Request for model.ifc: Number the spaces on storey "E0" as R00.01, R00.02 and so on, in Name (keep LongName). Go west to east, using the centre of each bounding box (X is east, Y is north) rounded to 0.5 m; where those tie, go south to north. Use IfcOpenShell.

First a look at what the model holds.

```python
import ifcopenshell
import ifcopenshell.util.element
import ifcopenshell.util.placement

model = ifcopenshell.open("model.ifc")
print(model.schema)
storey = next(s for s in model.by_type("IfcBuildingStorey") if s.Name == "E0")
spaces = [e for e in ifcopenshell.util.element.get_decomposition(storey) if e.is_a("IfcSpace")]
for e in sorted(spaces, key=lambda e: e.id()):
    origin = ifcopenshell.util.placement.get_local_placement(e.ObjectPlacement)[:3, 3]
    print(e.id(), e.Name, e.LongName, origin.round(2) + 0.0, sep=" | ")
```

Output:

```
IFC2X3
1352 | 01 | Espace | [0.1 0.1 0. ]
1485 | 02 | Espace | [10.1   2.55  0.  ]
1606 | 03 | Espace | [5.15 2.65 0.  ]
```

```python
import ifcopenshell
import ifcopenshell.geom
import ifcopenshell.util.element
import ifcopenshell.util.shape

model = ifcopenshell.open("model.ifc")
settings = ifcopenshell.geom.settings()
settings.set("use-world-coords", True)


def centre(element):
    shape = ifcopenshell.geom.create_shape(settings, element)
    return ifcopenshell.util.shape.get_bbox_centroid(shape.geometry)


storey = next(s for s in model.by_type("IfcBuildingStorey") if s.Name == "E0")
spaces = [e for e in ifcopenshell.util.element.get_decomposition(storey) if e.is_a("IfcSpace")]

# Insertion points can sit at a corner or the storey origin, so sort by the geometry (in metres).
centres = {e: centre(e) for e in spaces}
spaces.sort(key=lambda e: (round(centres[e][0] / 0.5), centres[e][1]))

for i, e in enumerate(spaces, start=1):
    number = f"R00.{i:02d}"
    e.Name = number
    print(e.id(), number)

model.write("model_edited.ifc")
```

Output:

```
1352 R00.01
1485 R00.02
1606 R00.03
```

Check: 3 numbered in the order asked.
